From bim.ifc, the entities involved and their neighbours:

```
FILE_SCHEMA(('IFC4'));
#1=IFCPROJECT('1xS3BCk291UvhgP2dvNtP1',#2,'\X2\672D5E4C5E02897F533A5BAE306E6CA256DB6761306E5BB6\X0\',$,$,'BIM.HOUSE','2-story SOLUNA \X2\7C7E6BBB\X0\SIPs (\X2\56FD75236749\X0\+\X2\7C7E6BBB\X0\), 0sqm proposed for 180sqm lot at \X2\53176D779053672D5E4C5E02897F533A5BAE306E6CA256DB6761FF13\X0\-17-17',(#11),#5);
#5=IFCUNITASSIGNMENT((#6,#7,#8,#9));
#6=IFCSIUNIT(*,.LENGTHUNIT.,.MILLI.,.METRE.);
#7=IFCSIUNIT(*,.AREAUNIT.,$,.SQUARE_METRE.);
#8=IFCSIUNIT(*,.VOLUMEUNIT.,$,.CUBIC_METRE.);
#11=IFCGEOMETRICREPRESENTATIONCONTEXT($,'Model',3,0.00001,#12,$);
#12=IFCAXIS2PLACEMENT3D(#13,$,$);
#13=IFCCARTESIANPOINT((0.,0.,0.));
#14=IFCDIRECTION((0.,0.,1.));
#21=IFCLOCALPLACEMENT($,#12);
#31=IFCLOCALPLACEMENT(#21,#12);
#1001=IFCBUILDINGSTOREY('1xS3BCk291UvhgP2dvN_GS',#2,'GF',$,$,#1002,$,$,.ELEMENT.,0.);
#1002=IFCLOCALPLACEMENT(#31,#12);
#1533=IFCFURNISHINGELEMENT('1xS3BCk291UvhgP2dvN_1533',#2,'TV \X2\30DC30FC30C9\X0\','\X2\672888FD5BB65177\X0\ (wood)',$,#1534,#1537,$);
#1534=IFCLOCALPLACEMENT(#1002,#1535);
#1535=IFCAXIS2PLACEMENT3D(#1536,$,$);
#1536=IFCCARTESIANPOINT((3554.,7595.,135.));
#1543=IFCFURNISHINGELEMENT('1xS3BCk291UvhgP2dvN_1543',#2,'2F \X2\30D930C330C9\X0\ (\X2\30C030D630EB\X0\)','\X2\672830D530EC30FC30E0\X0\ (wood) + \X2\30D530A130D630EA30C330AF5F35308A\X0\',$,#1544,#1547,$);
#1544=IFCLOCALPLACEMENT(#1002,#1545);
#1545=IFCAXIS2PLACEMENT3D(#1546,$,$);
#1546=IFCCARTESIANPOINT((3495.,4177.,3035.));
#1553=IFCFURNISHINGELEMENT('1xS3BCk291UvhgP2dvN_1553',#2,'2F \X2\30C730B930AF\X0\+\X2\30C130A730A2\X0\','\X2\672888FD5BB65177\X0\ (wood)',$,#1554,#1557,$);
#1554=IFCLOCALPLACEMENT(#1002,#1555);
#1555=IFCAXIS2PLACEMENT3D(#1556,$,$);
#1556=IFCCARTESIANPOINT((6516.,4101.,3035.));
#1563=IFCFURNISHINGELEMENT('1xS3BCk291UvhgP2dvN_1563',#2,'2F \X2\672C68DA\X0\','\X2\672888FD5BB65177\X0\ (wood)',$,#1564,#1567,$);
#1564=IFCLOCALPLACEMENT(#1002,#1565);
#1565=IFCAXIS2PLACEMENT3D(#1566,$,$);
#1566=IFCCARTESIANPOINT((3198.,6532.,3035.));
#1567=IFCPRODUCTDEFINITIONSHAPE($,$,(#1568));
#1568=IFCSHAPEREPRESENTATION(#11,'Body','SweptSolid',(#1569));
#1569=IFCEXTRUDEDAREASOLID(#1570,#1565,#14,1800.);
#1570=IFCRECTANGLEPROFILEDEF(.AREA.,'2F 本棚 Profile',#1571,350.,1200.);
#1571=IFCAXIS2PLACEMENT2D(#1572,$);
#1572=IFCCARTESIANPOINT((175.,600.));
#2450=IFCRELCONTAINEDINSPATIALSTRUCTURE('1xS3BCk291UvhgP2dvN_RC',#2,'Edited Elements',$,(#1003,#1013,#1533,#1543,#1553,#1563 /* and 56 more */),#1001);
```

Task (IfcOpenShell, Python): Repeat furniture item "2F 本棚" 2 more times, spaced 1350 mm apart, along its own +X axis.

```python
import ifcopenshell
import ifcopenshell.api.geometry
import ifcopenshell.api.root
import ifcopenshell.util.element
import ifcopenshell.util.placement
import ifcopenshell.util.unit

model = ifcopenshell.open("bim.ifc")
unit_scale = ifcopenshell.util.unit.calculate_unit_scale(model)


def reuse_history(source, copy):
    """copy_class also copies each property set's owner history, people and application; keep the originals."""
    for rel in copy.IsDefinedBy:
        if rel.is_a("IfcRelDefinesByProperties") and (history := rel.RelatingPropertyDefinition.OwnerHistory):
            rel.RelatingPropertyDefinition.OwnerHistory = source.OwnerHistory
            ifcopenshell.util.element.remove_deep2(model, history)


source = model.by_guid("1xS3BCk291UvhgP2dvN_1563")
base = ifcopenshell.util.placement.get_local_placement(source.ObjectPlacement)
step = base[:3, 0] * 1.35 / unit_scale

for i in range(1, 3):
    copy = ifcopenshell.api.root.copy_class(model, product=source)
    copy.Representation = ifcopenshell.util.element.copy_deep(
        model, source.Representation, exclude=["IfcGeometricRepresentationContext", "IfcRepresentationMap"]
    )
    reuse_history(source, copy)
    matrix = base.copy()
    matrix[:3, 3] += i * step
    print("added at", matrix[:3, 3].round(3) + 0.0)
    ifcopenshell.api.geometry.edit_object_placement(model, product=copy, matrix=matrix, is_si=False)

model.write("bim_updated.ifc")
```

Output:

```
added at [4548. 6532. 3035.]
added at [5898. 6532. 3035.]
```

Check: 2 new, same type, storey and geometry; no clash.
